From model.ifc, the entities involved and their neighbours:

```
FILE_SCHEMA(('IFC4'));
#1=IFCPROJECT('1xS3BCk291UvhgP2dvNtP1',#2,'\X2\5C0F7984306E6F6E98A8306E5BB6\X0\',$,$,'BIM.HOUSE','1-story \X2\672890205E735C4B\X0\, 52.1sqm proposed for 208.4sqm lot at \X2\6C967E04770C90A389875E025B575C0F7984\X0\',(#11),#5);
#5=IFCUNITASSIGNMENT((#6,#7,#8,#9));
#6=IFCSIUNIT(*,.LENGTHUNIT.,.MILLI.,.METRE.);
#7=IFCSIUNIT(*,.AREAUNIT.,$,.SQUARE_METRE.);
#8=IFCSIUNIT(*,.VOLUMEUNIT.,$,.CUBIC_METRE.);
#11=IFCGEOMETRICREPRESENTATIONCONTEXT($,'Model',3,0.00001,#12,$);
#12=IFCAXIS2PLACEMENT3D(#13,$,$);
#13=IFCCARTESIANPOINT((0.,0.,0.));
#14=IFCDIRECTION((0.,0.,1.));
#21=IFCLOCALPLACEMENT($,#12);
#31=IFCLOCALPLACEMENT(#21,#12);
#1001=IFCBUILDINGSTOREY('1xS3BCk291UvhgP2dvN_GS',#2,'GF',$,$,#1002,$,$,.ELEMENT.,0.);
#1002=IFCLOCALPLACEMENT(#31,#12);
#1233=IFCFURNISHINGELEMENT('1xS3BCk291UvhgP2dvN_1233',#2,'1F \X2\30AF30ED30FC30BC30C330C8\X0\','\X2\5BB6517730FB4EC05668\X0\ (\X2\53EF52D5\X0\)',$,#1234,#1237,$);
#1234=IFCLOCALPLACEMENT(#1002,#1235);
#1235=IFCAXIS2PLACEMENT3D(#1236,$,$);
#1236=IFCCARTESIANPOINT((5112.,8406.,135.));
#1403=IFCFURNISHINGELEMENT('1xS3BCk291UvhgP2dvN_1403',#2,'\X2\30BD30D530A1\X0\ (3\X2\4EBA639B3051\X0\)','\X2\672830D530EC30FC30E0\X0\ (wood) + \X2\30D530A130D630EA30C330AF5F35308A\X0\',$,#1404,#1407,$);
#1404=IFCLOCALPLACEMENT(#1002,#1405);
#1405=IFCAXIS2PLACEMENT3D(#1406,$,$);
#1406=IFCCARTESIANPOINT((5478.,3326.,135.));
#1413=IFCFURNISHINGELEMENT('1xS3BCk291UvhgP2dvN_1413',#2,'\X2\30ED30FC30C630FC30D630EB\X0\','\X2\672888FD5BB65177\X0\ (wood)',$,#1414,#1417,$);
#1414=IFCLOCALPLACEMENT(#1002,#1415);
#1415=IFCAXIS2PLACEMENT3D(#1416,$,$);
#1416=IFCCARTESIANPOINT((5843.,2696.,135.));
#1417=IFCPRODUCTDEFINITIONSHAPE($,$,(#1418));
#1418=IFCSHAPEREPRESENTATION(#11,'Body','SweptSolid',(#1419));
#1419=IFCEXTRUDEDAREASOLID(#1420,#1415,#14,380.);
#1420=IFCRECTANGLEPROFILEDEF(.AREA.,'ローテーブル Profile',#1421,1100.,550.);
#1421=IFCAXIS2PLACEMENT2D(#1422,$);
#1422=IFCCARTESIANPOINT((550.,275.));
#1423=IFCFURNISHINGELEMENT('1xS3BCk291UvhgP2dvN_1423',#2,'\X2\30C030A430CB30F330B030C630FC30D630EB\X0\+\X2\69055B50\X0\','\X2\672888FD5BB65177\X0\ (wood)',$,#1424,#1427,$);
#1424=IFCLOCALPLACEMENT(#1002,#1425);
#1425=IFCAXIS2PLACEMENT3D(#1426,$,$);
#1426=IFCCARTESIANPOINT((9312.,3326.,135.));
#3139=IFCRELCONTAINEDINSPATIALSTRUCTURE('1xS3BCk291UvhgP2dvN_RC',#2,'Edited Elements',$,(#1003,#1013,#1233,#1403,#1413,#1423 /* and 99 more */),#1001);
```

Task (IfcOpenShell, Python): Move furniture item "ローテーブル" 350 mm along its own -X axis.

```python
import ifcopenshell
import ifcopenshell.api.geometry
import ifcopenshell.util.placement
import ifcopenshell.util.unit

model = ifcopenshell.open("model.ifc")
unit_scale = ifcopenshell.util.unit.calculate_unit_scale(model)

item = model.by_guid("1xS3BCk291UvhgP2dvN_1413")
matrix = ifcopenshell.util.placement.get_local_placement(item.ObjectPlacement)
matrix[:3, 3] -= matrix[:3, 0] * 0.35 / unit_scale
ifcopenshell.api.geometry.edit_object_placement(model, product=item, matrix=matrix, is_si=False)

print(ifcopenshell.util.placement.get_local_placement(item.ObjectPlacement).round(3) + 0.0)

model.write("model-out.ifc")
```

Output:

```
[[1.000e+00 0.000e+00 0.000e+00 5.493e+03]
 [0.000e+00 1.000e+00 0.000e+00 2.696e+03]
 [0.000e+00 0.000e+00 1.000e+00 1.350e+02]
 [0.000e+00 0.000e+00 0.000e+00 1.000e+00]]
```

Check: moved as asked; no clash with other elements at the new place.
